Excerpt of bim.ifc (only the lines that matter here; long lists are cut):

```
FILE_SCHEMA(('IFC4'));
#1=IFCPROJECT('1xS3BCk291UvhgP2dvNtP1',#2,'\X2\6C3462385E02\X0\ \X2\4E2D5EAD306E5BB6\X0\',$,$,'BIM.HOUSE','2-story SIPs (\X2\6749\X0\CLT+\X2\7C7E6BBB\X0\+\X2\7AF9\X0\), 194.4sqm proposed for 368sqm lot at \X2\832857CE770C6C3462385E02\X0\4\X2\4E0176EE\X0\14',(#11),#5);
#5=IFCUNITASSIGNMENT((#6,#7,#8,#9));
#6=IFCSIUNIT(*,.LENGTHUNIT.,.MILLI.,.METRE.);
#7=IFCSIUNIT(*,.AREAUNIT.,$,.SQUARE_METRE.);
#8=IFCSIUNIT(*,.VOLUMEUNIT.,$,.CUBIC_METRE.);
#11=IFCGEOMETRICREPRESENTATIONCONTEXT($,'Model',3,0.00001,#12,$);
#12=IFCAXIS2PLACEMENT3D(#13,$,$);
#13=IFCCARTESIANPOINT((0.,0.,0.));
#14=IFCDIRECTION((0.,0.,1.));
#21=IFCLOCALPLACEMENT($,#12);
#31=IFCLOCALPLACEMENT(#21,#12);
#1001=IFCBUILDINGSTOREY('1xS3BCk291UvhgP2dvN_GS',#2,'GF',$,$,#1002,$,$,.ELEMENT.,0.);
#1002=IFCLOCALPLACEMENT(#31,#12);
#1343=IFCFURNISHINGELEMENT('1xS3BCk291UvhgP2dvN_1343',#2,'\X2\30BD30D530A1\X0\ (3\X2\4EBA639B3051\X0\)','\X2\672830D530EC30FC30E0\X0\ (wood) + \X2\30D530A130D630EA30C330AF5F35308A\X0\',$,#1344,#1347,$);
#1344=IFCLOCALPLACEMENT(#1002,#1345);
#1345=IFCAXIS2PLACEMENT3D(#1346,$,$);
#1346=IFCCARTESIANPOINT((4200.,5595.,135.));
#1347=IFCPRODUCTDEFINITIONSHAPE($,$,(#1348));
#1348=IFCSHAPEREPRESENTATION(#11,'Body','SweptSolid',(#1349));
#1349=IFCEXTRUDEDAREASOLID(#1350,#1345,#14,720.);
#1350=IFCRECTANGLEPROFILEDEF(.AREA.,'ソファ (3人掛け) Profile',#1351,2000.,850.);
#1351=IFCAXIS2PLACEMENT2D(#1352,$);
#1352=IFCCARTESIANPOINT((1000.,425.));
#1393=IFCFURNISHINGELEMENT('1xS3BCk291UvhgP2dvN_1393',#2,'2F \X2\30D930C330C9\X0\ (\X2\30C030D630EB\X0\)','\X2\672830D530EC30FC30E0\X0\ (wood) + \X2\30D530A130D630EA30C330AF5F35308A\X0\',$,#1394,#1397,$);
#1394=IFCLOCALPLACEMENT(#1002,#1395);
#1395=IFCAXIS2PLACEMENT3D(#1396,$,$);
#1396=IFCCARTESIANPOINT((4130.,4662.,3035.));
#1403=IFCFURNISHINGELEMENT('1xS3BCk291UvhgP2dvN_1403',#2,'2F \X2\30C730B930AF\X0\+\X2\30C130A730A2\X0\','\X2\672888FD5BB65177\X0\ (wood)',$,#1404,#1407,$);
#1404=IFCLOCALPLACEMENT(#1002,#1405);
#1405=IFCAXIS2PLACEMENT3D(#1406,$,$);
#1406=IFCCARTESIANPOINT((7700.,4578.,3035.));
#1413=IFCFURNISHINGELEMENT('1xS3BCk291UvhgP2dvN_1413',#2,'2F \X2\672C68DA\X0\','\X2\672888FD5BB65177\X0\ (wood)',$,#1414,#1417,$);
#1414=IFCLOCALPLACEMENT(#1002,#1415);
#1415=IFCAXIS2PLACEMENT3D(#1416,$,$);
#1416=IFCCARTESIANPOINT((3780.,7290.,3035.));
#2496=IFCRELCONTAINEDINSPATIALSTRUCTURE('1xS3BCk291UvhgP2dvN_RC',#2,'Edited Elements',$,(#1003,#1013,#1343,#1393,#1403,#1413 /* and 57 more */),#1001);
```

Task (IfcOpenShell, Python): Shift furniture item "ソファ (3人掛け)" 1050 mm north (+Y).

```python
import ifcopenshell
import ifcopenshell.api.geometry
import ifcopenshell.util.placement

model = ifcopenshell.open("bim.ifc")

item = model.by_guid("1xS3BCk291UvhgP2dvN_1343")
matrix = ifcopenshell.util.placement.get_local_placement(item.ObjectPlacement)
matrix[1, 3] += 1050.0
ifcopenshell.api.geometry.edit_object_placement(model, product=item, matrix=matrix, is_si=False)

print(ifcopenshell.util.placement.get_local_placement(item.ObjectPlacement).round(3) + 0.0)

model.write("bim_v2.ifc")
```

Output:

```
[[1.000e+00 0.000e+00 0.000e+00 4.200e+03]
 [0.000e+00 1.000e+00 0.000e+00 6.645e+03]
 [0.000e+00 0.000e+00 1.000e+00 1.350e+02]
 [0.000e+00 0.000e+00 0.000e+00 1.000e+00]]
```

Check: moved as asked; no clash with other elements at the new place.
